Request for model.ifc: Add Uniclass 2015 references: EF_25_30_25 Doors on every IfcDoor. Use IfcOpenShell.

First a look at what the model holds.

```python
import ifcopenshell

model = ifcopenshell.open("model.ifc")
print(model.schema)
print("classifications:", [c.Name for c in model.by_type("IfcClassification")])
for ifc_class in ("IfcDoor", "IfcRoof", "IfcStair", "IfcWall", "IfcWindow"):
    print(ifc_class, len(model.by_type(ifc_class)))
```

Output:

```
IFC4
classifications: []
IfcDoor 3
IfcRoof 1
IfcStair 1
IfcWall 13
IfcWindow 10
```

```python
import ifcopenshell
import ifcopenshell.api.classification

model = ifcopenshell.open("model.ifc")

system = ifcopenshell.api.classification.add_classification(model, classification="Uniclass 2015")

codes = {
    "IfcDoor": ("EF_25_30_25", "Doors"),
}
for ifc_class, (code, name) in codes.items():
    products = model.by_type(ifc_class)
    ifcopenshell.api.classification.add_reference(
        model, products=products, classification=system, identification=code, name=name
    )
    print(code, len(products))

model.write("model_rev.ifc")
```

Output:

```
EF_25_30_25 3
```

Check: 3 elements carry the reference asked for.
